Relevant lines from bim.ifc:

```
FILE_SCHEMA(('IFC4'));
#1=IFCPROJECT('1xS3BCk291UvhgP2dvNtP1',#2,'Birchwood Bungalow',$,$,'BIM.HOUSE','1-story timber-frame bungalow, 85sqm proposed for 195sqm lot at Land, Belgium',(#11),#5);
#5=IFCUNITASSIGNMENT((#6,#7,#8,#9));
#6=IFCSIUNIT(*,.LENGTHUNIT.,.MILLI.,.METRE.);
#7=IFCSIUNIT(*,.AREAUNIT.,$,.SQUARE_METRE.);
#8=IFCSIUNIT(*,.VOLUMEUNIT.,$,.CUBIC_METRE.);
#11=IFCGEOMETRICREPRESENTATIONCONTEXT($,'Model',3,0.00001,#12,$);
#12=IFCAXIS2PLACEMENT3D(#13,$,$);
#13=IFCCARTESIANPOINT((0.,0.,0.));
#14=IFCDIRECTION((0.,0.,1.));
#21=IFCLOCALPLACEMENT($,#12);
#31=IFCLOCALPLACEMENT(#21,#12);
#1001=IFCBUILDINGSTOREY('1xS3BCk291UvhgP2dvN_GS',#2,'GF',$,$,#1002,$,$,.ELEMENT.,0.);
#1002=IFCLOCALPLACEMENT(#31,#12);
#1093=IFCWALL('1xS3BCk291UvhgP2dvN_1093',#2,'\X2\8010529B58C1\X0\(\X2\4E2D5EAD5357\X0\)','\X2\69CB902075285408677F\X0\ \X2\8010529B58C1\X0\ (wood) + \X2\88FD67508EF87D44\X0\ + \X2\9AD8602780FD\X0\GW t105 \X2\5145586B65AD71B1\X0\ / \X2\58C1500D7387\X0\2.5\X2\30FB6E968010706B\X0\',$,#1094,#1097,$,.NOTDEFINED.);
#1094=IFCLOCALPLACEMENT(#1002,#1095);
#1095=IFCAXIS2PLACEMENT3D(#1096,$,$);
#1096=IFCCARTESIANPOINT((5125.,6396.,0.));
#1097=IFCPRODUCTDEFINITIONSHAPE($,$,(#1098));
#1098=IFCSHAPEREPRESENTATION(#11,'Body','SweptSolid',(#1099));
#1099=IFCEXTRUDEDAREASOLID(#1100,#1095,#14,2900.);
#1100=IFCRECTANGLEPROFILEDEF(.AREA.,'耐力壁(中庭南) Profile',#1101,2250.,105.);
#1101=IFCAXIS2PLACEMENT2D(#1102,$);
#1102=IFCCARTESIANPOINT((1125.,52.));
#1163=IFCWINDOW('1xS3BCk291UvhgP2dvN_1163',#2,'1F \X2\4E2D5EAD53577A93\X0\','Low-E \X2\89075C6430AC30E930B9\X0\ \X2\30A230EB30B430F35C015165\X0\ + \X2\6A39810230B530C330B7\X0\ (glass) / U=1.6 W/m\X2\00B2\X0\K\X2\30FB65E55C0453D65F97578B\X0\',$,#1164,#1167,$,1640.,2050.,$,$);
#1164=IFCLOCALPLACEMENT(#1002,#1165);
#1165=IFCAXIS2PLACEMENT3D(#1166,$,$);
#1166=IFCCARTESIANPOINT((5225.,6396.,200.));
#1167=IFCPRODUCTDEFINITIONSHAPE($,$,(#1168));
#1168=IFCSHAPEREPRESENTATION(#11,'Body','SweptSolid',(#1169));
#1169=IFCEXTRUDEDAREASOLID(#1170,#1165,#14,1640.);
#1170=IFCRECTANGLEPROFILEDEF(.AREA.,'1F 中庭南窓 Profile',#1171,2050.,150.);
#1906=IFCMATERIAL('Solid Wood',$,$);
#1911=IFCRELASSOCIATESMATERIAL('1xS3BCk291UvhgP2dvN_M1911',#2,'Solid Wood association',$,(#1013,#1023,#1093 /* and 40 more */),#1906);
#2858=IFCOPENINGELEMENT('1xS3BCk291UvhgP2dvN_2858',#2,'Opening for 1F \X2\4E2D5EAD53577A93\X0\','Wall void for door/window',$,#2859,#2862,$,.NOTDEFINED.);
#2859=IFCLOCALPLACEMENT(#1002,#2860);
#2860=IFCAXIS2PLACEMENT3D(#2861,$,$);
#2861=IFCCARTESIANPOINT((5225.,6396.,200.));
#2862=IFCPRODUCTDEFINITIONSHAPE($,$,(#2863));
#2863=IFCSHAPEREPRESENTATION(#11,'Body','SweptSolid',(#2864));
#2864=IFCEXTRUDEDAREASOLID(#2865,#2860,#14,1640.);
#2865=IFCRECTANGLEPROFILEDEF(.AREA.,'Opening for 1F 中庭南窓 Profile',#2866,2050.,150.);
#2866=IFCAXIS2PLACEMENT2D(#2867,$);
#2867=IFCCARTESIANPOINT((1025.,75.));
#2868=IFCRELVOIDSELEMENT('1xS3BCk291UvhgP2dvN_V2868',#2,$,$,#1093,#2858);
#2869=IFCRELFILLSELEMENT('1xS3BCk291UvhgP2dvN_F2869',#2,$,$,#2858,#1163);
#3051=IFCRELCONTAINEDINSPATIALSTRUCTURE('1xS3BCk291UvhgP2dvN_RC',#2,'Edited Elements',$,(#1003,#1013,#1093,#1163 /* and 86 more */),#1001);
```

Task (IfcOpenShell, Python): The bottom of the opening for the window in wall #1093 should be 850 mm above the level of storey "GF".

```python
import numpy as np
import ifcopenshell
import ifcopenshell.api.geometry
import ifcopenshell.geom
import ifcopenshell.util.element
import ifcopenshell.util.placement
import ifcopenshell.util.shape
import ifcopenshell.util.unit

model = ifcopenshell.open("bim.ifc")
unit_scale = ifcopenshell.util.unit.calculate_unit_scale(model)

window = model.by_id(1163)
opening = window.FillsVoids[0].RelatingOpeningElement
storey = ifcopenshell.util.element.get_container(window, ifc_class="IfcBuildingStorey")
level = ifcopenshell.util.placement.get_local_placement(storey.ObjectPlacement)[2, 3]

# The opening's origin need not be at the sill, so measure its lowest point.
shape = ifcopenshell.geom.create_shape(ifcopenshell.geom.settings(), opening)
bottom = ifcopenshell.util.shape.get_shape_bottom_elevation(shape, shape.geometry) / unit_scale
dz = level + 0.85 / unit_scale - bottom

shift = np.array([0.0, 0.0, dz])
# The window is not placed relative to its opening, so move both.
for product in (opening, window):
    matrix = ifcopenshell.util.placement.get_local_placement(product.ObjectPlacement)
    matrix[:3, 3] += shift
    ifcopenshell.api.geometry.edit_object_placement(model, product=product, matrix=matrix, is_si=False)

print(f"moved by {dz * unit_scale:+.3f} m")

model.write("bim_updated.ifc")
```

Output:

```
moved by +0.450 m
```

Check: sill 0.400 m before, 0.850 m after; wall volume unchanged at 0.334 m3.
